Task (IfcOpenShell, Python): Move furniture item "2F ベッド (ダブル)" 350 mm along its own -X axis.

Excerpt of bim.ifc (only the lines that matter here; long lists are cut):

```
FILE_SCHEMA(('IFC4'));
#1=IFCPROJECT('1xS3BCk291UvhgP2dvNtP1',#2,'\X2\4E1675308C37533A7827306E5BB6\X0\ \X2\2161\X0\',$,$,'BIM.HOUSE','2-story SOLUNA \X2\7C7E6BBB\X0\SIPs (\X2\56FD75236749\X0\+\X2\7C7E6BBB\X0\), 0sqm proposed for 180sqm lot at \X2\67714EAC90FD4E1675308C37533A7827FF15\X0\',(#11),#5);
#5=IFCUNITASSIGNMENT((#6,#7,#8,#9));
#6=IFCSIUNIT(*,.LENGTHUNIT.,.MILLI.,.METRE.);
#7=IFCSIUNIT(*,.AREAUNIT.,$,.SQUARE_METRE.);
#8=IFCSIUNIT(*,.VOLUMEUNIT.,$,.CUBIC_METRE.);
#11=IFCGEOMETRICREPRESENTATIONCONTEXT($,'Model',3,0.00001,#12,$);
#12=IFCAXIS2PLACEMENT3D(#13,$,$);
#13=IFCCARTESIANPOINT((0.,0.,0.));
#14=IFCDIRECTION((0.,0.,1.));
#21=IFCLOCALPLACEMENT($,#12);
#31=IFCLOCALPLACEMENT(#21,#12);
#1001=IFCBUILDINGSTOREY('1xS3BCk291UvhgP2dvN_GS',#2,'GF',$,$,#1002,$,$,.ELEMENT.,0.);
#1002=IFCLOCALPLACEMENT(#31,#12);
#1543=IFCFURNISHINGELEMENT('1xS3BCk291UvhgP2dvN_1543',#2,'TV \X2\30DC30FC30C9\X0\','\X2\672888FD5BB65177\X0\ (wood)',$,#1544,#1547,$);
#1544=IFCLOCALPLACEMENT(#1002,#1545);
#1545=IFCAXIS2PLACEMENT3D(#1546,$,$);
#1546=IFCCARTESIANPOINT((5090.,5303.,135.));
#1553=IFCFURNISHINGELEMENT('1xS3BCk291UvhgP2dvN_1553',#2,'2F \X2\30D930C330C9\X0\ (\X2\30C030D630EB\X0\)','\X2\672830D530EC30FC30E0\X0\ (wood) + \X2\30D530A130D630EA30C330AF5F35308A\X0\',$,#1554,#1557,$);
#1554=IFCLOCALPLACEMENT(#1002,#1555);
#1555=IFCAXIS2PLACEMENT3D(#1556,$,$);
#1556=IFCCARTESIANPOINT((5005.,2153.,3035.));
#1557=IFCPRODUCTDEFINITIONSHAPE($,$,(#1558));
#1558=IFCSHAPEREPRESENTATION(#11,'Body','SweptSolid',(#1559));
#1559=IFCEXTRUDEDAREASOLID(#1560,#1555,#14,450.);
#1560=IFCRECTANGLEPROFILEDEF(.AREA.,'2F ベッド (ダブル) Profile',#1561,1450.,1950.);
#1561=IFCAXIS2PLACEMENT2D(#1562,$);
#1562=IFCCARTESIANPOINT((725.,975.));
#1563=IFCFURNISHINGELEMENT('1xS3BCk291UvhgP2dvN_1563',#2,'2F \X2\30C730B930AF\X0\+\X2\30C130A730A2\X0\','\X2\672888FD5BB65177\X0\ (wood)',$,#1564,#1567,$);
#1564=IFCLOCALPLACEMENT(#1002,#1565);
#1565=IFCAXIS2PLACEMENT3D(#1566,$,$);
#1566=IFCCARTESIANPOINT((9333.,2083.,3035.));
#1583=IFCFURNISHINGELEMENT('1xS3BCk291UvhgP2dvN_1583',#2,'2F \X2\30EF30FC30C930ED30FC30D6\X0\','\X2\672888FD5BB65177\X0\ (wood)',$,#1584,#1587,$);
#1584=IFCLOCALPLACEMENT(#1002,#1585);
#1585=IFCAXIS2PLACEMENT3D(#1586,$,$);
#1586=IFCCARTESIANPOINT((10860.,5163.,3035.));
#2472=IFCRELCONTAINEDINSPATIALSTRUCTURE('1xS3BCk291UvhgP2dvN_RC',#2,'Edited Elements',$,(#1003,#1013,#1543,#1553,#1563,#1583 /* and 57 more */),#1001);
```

```python
import ifcopenshell
import ifcopenshell.api.geometry
import ifcopenshell.util.placement
import ifcopenshell.util.unit

model = ifcopenshell.open("bim.ifc")
unit_scale = ifcopenshell.util.unit.calculate_unit_scale(model)

item = model.by_guid("1xS3BCk291UvhgP2dvN_1553")
matrix = ifcopenshell.util.placement.get_local_placement(item.ObjectPlacement)
matrix[:3, 3] -= matrix[:3, 0] * 0.35 / unit_scale
ifcopenshell.api.geometry.edit_object_placement(model, product=item, matrix=matrix, is_si=False)

print(ifcopenshell.util.placement.get_local_placement(item.ObjectPlacement).round(3) + 0.0)

model.write("bim_updated.ifc")
```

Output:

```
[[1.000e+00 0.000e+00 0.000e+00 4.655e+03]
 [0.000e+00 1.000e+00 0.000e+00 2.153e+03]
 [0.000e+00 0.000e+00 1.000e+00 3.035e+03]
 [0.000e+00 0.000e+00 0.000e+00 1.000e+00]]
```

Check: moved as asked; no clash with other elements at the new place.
